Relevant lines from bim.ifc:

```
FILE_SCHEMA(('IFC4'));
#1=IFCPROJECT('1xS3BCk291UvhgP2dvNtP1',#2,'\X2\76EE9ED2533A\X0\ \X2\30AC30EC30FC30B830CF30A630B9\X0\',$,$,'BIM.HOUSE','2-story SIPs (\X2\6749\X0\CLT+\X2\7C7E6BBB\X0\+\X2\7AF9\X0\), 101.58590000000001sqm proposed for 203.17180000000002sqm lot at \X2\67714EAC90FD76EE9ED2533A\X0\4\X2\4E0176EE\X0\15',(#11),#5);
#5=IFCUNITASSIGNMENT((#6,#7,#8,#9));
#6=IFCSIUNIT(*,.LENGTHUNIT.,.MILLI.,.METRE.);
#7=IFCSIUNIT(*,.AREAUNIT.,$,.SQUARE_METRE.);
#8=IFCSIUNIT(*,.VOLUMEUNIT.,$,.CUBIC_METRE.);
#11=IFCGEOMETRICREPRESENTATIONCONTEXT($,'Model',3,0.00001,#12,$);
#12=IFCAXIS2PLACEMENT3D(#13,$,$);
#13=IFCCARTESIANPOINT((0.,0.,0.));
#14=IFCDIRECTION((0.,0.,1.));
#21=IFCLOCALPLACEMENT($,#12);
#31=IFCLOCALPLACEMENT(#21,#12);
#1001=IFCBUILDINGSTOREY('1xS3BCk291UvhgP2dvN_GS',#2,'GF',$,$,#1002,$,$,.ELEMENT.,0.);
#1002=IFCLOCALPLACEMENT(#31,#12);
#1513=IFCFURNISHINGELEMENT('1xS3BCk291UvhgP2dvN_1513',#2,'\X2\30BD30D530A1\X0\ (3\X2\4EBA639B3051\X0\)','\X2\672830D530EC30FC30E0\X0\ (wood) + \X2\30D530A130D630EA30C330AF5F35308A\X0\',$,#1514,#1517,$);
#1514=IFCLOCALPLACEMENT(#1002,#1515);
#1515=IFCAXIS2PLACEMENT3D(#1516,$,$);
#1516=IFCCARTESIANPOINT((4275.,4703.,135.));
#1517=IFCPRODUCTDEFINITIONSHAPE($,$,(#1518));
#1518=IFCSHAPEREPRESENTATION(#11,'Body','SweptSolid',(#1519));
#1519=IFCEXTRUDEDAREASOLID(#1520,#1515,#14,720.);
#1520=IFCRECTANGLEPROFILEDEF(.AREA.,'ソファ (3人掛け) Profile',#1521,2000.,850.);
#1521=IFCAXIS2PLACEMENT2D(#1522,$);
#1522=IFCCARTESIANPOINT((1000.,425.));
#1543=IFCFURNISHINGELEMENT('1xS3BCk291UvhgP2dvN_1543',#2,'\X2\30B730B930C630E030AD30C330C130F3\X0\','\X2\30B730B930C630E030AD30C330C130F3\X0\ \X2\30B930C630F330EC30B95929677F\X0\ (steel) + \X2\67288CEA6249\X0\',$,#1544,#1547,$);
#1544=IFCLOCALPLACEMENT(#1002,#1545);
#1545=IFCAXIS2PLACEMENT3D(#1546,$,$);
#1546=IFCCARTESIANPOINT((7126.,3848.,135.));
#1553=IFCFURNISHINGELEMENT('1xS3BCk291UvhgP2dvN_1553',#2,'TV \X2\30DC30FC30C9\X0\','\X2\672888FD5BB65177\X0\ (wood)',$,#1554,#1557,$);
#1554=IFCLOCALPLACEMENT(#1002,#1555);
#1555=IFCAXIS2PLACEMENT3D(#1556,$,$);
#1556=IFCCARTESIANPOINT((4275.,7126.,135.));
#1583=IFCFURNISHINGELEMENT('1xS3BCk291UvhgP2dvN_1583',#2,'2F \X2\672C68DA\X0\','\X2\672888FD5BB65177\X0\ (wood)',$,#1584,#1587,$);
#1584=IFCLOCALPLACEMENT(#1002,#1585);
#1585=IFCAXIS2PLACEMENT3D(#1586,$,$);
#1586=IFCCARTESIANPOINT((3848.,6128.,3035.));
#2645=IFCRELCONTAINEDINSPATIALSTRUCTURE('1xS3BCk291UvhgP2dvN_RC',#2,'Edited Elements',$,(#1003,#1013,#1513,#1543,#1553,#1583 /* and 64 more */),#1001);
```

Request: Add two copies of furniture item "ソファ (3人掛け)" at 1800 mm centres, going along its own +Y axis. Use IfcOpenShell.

```python
import ifcopenshell
import ifcopenshell.api.geometry
import ifcopenshell.api.root
import ifcopenshell.util.element
import ifcopenshell.util.placement

model = ifcopenshell.open("bim.ifc")


def reuse_history(source, copy):
    """copy_class also copies each property set's owner history, people and application; keep the originals."""
    for rel in copy.IsDefinedBy:
        if rel.is_a("IfcRelDefinesByProperties") and (history := rel.RelatingPropertyDefinition.OwnerHistory):
            rel.RelatingPropertyDefinition.OwnerHistory = source.OwnerHistory
            ifcopenshell.util.element.remove_deep2(model, history)


source = model.by_guid("1xS3BCk291UvhgP2dvN_1513")
base = ifcopenshell.util.placement.get_local_placement(source.ObjectPlacement)
step = base[:3, 1] * 1800.0

for i in range(1, 3):
    copy = ifcopenshell.api.root.copy_class(model, product=source)
    copy.Representation = ifcopenshell.util.element.copy_deep(
        model, source.Representation, exclude=["IfcGeometricRepresentationContext", "IfcRepresentationMap"]
    )
    reuse_history(source, copy)
    matrix = base.copy()
    matrix[:3, 3] += i * step
    print("added at", matrix[:3, 3].round(3) + 0.0)
    ifcopenshell.api.geometry.edit_object_placement(model, product=copy, matrix=matrix, is_si=False)

model.write("bim_rev.ifc")
```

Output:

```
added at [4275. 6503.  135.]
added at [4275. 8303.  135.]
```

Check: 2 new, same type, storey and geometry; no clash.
